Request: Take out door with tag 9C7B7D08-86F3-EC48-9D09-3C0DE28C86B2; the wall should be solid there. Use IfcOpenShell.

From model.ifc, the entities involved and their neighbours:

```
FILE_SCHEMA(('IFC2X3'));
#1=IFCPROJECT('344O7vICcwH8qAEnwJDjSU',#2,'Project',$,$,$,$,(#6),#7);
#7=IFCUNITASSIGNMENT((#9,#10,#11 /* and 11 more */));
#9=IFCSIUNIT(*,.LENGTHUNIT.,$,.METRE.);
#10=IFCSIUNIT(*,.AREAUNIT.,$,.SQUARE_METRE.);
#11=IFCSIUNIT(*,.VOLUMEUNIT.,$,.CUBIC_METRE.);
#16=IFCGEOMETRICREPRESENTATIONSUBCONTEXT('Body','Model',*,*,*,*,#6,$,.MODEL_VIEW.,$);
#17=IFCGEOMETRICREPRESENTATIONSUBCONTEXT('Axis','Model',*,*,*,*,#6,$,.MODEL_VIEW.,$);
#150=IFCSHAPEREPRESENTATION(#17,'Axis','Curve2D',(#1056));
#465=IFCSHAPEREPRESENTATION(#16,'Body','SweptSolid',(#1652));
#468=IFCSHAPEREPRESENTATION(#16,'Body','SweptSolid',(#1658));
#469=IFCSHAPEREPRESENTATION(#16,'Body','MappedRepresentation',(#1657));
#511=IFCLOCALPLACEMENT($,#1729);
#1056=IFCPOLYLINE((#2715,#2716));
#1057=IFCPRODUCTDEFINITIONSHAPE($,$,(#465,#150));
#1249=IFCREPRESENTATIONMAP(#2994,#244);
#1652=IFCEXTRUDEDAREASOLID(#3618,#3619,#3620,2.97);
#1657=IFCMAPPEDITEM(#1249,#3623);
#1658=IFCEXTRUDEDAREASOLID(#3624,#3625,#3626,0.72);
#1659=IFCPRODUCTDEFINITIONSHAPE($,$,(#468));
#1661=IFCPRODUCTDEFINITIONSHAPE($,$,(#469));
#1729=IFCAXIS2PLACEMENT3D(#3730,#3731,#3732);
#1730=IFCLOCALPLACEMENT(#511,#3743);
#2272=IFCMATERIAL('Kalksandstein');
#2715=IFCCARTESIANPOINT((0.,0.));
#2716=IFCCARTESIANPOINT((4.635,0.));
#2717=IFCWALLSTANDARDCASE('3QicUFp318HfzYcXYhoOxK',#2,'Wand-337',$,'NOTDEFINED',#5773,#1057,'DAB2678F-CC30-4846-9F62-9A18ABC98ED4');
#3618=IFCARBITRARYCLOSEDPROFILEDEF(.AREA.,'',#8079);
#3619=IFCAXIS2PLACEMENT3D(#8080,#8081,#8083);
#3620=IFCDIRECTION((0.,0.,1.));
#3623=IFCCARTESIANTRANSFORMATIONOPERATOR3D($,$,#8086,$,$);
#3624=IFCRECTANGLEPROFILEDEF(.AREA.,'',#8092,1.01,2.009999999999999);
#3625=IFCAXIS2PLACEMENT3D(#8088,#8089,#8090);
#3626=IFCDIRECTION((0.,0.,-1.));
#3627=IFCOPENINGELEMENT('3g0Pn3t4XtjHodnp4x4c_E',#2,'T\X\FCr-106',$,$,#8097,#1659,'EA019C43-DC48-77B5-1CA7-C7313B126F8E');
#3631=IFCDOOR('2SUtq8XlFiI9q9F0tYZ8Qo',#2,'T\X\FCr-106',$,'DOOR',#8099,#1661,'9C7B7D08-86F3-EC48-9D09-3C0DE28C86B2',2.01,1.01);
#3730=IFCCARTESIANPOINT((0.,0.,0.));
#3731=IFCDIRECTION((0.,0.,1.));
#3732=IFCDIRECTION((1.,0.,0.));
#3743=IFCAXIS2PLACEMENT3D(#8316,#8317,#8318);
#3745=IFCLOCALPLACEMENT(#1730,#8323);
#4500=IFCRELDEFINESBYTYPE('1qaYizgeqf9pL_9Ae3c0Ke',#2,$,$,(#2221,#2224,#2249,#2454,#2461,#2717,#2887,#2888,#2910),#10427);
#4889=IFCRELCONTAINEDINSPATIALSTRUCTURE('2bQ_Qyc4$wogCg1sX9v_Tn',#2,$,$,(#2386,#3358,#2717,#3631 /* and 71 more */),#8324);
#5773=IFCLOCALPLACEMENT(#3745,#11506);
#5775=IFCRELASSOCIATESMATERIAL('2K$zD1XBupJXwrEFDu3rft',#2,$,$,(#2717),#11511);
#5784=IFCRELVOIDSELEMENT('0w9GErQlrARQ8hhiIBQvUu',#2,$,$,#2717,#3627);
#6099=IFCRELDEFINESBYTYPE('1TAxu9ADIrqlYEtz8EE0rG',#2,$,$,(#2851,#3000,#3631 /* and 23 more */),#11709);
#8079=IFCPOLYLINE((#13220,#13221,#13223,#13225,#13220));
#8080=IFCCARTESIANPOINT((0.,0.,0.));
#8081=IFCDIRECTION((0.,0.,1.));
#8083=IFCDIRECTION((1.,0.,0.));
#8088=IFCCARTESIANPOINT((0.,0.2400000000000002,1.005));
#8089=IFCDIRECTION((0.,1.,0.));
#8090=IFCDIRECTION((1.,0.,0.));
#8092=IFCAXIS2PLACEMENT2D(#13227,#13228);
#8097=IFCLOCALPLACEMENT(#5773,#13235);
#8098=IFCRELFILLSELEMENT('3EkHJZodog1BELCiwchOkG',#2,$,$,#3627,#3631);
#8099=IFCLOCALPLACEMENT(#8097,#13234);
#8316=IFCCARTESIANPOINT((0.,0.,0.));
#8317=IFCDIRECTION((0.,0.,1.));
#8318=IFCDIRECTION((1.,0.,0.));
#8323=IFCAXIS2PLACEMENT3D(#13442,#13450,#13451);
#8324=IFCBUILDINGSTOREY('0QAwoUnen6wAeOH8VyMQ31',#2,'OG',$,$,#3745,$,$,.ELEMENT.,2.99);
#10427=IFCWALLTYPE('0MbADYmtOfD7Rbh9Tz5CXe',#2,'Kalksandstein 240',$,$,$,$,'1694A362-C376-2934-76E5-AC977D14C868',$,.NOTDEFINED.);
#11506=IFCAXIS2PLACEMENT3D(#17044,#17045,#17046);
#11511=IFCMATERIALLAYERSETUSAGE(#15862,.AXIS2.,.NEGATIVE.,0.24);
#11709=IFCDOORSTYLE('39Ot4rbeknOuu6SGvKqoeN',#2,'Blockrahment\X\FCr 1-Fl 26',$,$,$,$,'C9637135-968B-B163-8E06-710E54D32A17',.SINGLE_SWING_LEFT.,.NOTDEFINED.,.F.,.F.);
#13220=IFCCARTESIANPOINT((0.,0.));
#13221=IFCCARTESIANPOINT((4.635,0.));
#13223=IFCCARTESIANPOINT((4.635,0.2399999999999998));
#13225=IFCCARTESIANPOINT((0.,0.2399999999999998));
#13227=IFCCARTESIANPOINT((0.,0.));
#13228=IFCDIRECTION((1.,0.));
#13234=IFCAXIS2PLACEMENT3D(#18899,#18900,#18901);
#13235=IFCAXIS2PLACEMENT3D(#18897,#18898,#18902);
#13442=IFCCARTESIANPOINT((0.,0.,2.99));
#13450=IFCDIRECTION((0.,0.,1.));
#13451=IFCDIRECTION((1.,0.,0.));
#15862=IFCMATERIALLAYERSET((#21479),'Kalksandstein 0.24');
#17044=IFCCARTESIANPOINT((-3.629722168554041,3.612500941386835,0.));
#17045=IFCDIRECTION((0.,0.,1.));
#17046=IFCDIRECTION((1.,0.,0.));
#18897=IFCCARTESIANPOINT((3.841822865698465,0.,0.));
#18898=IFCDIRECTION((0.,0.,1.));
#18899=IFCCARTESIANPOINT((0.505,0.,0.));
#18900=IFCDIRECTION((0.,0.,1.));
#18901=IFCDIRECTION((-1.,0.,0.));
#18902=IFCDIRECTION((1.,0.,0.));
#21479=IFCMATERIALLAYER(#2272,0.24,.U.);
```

```python
import ifcopenshell
import ifcopenshell.api.feature
import ifcopenshell.api.root
import ifcopenshell.geom
import ifcopenshell.util.shape

model = ifcopenshell.open("model.ifc")
settings = ifcopenshell.geom.settings()


def volume(element):
    """Net volume in cubic metres, openings subtracted."""
    shape = ifcopenshell.geom.create_shape(settings, element)
    return ifcopenshell.util.shape.get_volume(shape.geometry)


door = model.by_guid("2SUtq8XlFiI9q9F0tYZ8Qo")
opening = door.FillsVoids[0].RelatingOpeningElement
wall = opening.VoidsElements[0].RelatingBuildingElement
before = volume(wall)

ifcopenshell.api.root.remove_product(model, product=door)
ifcopenshell.api.feature.remove_feature(model, feature=opening)

after = volume(wall)

print(f"wall volume {before:.3f} -> {after:.3f} m3")

model.write("model_edited.ifc")
```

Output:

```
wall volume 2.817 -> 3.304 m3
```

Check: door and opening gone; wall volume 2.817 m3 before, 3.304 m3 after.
